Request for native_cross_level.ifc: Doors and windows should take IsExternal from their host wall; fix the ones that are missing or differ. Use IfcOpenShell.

First a look at what the model holds.

```python
import ifcopenshell
import ifcopenshell.util.element

model = ifcopenshell.open("native_cross_level.ifc")
print(model.schema)
seen = {}
for e in model.by_type("IfcDoor") + model.by_type("IfcWindow"):
    if not e.FillsVoids:
        continue
    host = e.FillsVoids[0].RelatingOpeningElement.VoidsElements[0].RelatingBuildingElement
    own = ifcopenshell.util.element.get_pset(e, f"Pset_{e.is_a()[3:].removesuffix('StandardCase')}Common", "IsExternal")
    wall = ifcopenshell.util.element.get_pset(host, "Pset_WallCommon", "IsExternal")
    seen[e.is_a(), own, wall] = seen.get((e.is_a(), own, wall), 0) + 1
for (cls, own, wall), count in sorted(seen.items(), key=str):
    print(count, cls, "IsExternal:", own, "| host wall:", wall)
```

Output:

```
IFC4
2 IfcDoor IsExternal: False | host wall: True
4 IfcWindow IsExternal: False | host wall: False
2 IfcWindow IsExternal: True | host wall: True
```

```python
import ifcopenshell
import ifcopenshell.api.pset
import ifcopenshell.util.element

model = ifcopenshell.open("native_cross_level.ifc")

count = 0
for ifc_class, pset_name in (("IfcDoor", "Pset_DoorCommon"), ("IfcWindow", "Pset_WindowCommon")):
    for e in model.by_type(ifc_class):
        if not e.FillsVoids:
            continue
        host = e.FillsVoids[0].RelatingOpeningElement.VoidsElements[0].RelatingBuildingElement
        external = ifcopenshell.util.element.get_pset(host, "Pset_WallCommon", "IsExternal")
        if external is None or ifcopenshell.util.element.get_pset(e, pset_name, "IsExternal") == external:
            continue
        pset = ifcopenshell.api.pset.add_pset(model, product=e, name=pset_name)
        ifcopenshell.api.pset.edit_pset(model, pset=pset, properties={"IsExternal": external})
        count += 1

print(count, "updated")

model.write("native_cross_level_v2.ifc")
```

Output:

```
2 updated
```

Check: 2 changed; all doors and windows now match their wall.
